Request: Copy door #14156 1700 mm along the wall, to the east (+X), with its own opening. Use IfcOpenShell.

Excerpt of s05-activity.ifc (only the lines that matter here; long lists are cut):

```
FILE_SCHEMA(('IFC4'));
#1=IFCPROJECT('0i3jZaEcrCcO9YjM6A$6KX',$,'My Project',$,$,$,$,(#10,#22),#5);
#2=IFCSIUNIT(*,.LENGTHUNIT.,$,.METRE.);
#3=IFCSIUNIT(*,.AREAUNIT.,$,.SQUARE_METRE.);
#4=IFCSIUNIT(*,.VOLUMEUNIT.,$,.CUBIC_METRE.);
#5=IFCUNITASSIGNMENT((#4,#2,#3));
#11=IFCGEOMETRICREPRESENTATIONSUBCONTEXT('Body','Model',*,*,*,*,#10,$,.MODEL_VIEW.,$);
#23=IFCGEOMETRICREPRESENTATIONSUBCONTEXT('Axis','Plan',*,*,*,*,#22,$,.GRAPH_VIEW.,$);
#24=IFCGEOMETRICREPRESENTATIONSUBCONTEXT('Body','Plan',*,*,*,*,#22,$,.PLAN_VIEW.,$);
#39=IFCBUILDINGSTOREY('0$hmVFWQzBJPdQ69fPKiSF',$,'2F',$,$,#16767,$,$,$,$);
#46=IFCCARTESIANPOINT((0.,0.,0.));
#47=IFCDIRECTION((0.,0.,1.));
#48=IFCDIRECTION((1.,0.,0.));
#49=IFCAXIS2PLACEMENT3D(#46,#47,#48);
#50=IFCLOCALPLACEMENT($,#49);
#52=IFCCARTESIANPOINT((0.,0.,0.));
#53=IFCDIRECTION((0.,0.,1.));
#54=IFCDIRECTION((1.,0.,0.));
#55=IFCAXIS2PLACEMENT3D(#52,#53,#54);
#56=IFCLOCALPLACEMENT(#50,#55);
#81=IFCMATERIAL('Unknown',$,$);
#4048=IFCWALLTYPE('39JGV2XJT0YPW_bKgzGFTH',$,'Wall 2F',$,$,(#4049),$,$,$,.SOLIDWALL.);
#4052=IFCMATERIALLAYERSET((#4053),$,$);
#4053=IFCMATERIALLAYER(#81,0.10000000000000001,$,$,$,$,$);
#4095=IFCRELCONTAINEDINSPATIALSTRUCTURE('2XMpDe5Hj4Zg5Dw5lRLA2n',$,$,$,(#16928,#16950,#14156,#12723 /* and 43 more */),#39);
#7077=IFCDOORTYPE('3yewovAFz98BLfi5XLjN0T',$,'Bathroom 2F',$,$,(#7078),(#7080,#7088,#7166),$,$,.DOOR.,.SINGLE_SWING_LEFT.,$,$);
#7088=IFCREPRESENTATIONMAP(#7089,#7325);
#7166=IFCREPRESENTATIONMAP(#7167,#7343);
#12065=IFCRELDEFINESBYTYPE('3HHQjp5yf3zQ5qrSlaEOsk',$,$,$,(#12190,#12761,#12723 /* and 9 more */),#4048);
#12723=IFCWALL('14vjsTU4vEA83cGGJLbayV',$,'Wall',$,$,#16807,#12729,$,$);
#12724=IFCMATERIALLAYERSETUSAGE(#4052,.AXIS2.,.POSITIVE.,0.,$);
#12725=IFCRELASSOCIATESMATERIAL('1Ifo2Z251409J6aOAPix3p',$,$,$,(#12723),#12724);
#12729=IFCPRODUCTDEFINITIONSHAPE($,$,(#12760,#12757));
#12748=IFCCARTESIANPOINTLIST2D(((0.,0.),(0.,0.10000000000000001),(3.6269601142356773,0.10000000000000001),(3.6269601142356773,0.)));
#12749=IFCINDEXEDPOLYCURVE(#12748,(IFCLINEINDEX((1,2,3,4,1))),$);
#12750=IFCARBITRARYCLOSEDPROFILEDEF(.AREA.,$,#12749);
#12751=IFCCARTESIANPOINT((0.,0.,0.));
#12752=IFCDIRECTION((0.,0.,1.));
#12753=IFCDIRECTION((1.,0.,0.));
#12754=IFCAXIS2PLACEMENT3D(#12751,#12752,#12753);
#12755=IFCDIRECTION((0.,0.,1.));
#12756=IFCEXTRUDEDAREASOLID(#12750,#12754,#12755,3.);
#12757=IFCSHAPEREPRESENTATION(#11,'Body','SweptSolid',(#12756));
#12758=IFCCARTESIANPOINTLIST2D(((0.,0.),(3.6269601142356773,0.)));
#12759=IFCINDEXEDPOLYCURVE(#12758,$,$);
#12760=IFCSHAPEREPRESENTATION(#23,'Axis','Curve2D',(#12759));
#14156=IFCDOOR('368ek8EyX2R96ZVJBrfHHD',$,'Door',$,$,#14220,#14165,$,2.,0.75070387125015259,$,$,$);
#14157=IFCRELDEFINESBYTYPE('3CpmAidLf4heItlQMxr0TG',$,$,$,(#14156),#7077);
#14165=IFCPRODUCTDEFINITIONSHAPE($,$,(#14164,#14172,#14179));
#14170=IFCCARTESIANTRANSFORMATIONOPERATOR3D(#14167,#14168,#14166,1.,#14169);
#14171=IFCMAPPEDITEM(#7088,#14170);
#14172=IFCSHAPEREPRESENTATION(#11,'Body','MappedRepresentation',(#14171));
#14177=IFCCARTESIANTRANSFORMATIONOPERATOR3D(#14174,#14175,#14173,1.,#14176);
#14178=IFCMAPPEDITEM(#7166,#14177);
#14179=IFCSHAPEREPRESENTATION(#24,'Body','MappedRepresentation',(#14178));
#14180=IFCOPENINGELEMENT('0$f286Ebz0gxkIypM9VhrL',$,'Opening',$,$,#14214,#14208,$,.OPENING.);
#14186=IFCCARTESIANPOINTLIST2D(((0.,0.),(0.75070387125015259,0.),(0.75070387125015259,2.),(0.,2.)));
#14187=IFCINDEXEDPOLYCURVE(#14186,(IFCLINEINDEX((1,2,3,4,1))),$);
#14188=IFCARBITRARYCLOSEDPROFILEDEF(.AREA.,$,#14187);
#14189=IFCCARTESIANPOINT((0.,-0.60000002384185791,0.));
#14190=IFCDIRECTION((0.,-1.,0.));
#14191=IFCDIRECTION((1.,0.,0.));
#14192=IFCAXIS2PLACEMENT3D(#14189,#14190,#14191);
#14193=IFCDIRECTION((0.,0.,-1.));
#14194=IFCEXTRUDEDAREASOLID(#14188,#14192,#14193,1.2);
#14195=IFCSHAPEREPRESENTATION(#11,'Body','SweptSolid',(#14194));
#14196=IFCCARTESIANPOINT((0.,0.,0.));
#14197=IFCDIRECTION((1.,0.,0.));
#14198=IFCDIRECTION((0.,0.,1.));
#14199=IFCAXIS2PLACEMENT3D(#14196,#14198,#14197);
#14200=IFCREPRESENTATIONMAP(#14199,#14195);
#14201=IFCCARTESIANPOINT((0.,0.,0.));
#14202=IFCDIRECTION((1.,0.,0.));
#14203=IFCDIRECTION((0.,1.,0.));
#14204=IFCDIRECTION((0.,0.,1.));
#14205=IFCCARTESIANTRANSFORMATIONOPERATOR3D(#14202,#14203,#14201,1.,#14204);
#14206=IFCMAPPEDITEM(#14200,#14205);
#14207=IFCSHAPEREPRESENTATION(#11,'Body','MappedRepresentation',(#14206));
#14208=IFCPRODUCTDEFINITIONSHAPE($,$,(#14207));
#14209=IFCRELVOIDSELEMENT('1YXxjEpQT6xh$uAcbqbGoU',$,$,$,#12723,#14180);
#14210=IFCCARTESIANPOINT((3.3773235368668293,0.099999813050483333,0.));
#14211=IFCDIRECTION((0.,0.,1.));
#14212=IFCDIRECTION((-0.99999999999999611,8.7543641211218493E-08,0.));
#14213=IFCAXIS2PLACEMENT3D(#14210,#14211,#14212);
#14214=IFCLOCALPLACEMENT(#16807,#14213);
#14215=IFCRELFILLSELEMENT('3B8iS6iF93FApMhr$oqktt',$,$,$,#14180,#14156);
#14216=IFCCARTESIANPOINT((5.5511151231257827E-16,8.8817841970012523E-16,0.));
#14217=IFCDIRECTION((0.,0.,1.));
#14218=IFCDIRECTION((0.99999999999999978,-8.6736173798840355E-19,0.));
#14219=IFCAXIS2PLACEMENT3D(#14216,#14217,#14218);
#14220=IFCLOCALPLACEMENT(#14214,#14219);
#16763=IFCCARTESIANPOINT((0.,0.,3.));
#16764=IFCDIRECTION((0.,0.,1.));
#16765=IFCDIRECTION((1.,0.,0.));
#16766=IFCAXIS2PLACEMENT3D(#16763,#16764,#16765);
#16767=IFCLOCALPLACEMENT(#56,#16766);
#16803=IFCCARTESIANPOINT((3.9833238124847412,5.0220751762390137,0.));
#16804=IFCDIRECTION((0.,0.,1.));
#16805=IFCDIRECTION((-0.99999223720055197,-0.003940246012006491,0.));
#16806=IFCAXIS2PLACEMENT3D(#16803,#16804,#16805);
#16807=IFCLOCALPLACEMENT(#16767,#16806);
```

```python
import ifcopenshell
import ifcopenshell.api.feature
import ifcopenshell.api.geometry
import ifcopenshell.api.root
import ifcopenshell.geom
import ifcopenshell.util.element
import ifcopenshell.util.placement
import ifcopenshell.util.shape
import ifcopenshell.util.unit

model = ifcopenshell.open("s05-activity.ifc")
unit_scale = ifcopenshell.util.unit.calculate_unit_scale(model)
settings = ifcopenshell.geom.settings()


def volume(element):
    """Net volume in cubic metres, openings subtracted."""
    shape = ifcopenshell.geom.create_shape(settings, element)
    return ifcopenshell.util.shape.get_volume(shape.geometry)


door = model.by_guid("368ek8EyX2R96ZVJBrfHHD")
opening = door.FillsVoids[0].RelatingOpeningElement
wall = opening.VoidsElements[0].RelatingBuildingElement
before = volume(wall)
shift = ifcopenshell.util.placement.get_local_placement(wall.ObjectPlacement)[:3, 0] * -1.7 / unit_scale

# copy_class copies the void relationship, type, container and properties, but no geometry.
new_opening = ifcopenshell.api.root.copy_class(model, product=opening)
new_opening.Representation = ifcopenshell.util.element.copy_deep(
    model, opening.Representation, exclude=["IfcGeometricRepresentationContext", "IfcRepresentationMap"]
)
new_door = ifcopenshell.api.root.copy_class(model, product=door)
new_door.Representation = ifcopenshell.util.element.copy_deep(
    model, door.Representation, exclude=["IfcGeometricRepresentationContext", "IfcRepresentationMap"]
)
ifcopenshell.api.feature.add_filling(model, opening=new_opening, element=new_door)

for old, new in ((opening, new_opening), (door, new_door)):
    matrix = ifcopenshell.util.placement.get_local_placement(old.ObjectPlacement)
    matrix[:3, 3] += shift
    ifcopenshell.api.geometry.edit_object_placement(model, product=new, matrix=matrix, is_si=False)

after = volume(wall)

print(f"wall volume {before:.3f} -> {after:.3f} m3")

model.write("s05-activity_updated.ifc")
```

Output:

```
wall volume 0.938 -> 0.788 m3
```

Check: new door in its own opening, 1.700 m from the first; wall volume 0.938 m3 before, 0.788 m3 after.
